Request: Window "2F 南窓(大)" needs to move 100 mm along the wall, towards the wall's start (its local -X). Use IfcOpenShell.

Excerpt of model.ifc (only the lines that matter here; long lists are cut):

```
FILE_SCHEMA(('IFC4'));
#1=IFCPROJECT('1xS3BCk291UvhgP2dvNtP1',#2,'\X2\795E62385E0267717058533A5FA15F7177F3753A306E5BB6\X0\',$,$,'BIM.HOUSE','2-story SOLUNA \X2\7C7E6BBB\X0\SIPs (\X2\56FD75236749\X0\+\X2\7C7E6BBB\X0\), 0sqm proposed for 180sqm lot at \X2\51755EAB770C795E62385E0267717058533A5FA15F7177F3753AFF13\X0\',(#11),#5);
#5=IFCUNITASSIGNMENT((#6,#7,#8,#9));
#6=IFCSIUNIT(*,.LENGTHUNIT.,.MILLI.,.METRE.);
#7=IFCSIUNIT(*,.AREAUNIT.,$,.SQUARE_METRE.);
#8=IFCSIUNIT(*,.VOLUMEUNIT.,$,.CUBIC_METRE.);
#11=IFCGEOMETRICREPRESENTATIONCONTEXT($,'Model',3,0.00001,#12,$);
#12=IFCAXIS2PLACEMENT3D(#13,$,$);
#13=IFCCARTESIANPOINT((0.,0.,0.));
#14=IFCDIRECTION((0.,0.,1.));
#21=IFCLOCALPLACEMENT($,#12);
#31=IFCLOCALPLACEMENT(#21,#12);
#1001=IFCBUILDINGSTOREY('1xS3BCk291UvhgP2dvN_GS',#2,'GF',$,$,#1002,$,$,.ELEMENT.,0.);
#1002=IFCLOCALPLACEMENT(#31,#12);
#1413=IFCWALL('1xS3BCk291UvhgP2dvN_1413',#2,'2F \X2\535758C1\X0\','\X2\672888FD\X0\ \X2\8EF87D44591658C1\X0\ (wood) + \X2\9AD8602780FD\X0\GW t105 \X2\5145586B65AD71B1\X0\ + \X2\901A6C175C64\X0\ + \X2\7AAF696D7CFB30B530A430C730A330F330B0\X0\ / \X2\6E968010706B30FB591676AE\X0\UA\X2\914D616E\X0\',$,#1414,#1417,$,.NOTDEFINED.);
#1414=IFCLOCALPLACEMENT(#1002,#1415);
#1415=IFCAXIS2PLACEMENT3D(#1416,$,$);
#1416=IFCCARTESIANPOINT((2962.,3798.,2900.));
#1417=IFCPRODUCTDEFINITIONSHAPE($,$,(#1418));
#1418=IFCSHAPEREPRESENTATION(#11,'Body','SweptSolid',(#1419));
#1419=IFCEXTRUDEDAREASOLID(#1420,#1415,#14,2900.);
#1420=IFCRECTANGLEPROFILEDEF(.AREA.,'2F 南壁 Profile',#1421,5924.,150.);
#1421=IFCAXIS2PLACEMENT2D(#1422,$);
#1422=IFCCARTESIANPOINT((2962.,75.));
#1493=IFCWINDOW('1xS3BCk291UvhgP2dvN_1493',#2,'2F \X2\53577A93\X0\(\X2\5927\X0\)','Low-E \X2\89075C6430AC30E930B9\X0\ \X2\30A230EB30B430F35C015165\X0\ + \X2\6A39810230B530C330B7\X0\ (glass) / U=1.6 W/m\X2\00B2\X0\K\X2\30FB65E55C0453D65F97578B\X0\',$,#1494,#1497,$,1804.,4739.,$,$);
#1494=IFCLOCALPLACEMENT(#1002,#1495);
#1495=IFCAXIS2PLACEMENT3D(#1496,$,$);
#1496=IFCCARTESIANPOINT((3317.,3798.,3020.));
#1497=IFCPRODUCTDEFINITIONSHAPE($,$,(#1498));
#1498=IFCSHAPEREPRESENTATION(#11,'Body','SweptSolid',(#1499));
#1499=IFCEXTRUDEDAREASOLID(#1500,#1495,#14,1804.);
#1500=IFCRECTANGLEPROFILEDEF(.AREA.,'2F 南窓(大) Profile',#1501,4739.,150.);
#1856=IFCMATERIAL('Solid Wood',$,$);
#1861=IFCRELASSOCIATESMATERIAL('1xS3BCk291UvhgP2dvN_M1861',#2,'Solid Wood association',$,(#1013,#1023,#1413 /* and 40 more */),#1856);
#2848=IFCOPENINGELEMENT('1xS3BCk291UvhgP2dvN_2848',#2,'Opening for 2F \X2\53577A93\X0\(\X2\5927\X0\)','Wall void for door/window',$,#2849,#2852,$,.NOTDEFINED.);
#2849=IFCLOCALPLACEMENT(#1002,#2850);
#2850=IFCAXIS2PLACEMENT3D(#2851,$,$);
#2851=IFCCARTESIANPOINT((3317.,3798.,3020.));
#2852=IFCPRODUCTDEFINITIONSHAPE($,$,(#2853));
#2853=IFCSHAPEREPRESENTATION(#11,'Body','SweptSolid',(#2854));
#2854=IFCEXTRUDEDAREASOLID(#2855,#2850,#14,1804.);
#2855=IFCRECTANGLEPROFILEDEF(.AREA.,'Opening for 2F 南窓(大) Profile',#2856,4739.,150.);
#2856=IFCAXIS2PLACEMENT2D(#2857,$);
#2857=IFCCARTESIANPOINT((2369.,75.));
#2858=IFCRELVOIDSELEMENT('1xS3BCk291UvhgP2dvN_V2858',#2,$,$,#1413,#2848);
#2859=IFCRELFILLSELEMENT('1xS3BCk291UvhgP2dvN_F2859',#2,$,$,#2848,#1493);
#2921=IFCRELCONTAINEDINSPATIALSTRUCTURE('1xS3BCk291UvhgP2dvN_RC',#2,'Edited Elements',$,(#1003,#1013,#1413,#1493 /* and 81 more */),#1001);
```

```python
import ifcopenshell
import ifcopenshell.api.geometry
import ifcopenshell.util.placement
import ifcopenshell.util.unit

model = ifcopenshell.open("model.ifc")
unit_scale = ifcopenshell.util.unit.calculate_unit_scale(model)

window = model.by_guid("1xS3BCk291UvhgP2dvN_1493")
opening = window.FillsVoids[0].RelatingOpeningElement
wall = opening.VoidsElements[0].RelatingBuildingElement

wall_matrix = ifcopenshell.util.placement.get_local_placement(wall.ObjectPlacement)
shift = wall_matrix[:3, 0] * -0.1 / unit_scale
before = ifcopenshell.util.placement.get_local_placement(window.ObjectPlacement)[:3, 3].copy()

# The window is not placed relative to its opening, so move both.
for product in (opening, window):
    matrix = ifcopenshell.util.placement.get_local_placement(product.ObjectPlacement)
    matrix[:3, 3] += shift
    ifcopenshell.api.geometry.edit_object_placement(model, product=product, matrix=matrix, is_si=False)

after = ifcopenshell.util.placement.get_local_placement(window.ObjectPlacement)[:3, 3]
print("window moved by", (after - before).round(3) + 0.0)

model.write("model-out.ifc")
```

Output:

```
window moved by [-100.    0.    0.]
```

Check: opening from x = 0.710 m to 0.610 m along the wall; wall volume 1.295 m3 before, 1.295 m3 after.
